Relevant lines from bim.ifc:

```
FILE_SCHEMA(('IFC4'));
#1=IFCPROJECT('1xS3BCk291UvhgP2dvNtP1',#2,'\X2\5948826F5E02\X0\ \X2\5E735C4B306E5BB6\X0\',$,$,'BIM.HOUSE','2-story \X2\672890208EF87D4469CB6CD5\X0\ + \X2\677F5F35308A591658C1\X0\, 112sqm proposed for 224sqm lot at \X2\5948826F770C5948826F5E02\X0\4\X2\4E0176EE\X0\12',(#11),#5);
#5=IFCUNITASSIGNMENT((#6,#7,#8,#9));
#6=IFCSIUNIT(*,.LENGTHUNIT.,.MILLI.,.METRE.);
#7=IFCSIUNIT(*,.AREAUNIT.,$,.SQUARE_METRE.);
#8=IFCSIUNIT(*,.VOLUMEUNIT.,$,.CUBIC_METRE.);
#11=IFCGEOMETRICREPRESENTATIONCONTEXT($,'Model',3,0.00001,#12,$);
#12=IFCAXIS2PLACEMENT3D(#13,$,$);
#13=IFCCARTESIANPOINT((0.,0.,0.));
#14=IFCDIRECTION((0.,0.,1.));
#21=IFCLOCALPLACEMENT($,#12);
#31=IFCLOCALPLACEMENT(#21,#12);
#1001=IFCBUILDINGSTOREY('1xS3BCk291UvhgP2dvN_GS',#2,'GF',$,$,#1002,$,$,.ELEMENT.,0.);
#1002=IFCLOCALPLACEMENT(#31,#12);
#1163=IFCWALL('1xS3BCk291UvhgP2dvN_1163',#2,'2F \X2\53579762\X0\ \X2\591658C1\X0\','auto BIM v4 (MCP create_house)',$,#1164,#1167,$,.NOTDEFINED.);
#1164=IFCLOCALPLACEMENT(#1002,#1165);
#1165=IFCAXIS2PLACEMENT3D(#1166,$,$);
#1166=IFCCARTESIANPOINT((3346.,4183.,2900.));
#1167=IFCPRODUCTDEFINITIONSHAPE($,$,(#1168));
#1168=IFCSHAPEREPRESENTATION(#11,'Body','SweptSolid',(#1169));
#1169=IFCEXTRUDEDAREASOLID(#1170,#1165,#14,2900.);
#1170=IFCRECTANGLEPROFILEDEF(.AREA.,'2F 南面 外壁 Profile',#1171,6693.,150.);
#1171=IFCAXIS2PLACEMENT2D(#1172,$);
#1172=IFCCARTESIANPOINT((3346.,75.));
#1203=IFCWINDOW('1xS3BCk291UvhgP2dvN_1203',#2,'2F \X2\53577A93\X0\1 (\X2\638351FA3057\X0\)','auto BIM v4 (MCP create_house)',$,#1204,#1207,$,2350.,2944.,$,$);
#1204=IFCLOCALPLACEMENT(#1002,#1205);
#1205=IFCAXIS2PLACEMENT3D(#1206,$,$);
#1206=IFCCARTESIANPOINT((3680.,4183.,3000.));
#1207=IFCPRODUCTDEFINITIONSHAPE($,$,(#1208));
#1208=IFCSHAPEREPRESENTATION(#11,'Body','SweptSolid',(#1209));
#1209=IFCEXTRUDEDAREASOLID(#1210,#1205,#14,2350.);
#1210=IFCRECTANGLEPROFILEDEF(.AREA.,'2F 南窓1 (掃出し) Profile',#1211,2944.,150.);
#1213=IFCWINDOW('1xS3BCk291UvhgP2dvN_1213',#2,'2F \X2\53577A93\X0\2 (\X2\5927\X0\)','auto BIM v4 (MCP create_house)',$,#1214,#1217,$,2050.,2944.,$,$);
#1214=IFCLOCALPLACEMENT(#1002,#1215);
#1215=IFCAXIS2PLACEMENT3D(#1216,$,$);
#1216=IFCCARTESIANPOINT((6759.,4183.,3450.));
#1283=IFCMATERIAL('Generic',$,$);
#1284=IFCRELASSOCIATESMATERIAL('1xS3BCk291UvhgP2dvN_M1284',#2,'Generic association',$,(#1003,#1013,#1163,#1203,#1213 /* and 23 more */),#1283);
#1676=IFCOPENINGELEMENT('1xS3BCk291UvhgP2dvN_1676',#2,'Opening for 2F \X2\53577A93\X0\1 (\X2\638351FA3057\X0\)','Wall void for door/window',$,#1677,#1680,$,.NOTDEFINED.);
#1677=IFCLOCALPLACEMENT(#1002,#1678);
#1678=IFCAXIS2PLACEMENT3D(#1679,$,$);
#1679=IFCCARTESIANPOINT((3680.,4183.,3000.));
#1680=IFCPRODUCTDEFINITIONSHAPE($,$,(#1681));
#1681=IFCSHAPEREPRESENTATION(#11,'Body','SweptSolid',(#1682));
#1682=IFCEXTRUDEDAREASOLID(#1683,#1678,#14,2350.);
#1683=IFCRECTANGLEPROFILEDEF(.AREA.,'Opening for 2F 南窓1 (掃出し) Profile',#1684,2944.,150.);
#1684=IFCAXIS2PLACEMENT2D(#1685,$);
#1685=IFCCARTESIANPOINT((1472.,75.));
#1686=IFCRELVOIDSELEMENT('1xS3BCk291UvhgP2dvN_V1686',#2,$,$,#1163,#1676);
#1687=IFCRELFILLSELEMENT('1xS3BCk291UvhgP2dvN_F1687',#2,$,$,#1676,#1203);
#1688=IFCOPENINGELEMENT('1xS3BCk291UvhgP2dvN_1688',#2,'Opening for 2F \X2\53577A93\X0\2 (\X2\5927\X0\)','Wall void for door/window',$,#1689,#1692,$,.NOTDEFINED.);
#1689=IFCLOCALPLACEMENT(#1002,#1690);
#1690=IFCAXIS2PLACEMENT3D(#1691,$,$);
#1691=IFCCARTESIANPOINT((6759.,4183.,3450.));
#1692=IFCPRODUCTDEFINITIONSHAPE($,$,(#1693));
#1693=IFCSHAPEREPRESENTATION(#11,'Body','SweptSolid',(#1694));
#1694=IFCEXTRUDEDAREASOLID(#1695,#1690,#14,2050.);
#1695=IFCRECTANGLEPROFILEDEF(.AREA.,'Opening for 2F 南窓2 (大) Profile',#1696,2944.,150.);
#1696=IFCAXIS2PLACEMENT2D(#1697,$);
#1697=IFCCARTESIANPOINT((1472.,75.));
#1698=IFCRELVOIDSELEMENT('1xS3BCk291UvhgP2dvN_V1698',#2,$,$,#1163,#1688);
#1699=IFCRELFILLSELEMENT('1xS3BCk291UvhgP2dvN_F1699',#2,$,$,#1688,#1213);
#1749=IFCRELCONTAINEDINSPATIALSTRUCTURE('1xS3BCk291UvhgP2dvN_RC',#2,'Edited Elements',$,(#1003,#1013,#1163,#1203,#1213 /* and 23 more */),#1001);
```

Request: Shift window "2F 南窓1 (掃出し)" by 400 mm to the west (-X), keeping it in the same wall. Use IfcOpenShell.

```python
import ifcopenshell
import ifcopenshell.api.geometry
import ifcopenshell.util.placement
import ifcopenshell.util.unit

model = ifcopenshell.open("bim.ifc")
unit_scale = ifcopenshell.util.unit.calculate_unit_scale(model)

window = model.by_guid("1xS3BCk291UvhgP2dvN_1203")
opening = window.FillsVoids[0].RelatingOpeningElement
wall = opening.VoidsElements[0].RelatingBuildingElement

wall_matrix = ifcopenshell.util.placement.get_local_placement(wall.ObjectPlacement)
shift = wall_matrix[:3, 0] * -0.4 / unit_scale
before = ifcopenshell.util.placement.get_local_placement(window.ObjectPlacement)[:3, 3].copy()

# The window is not placed relative to its opening, so move both.
for product in (opening, window):
    matrix = ifcopenshell.util.placement.get_local_placement(product.ObjectPlacement)
    matrix[:3, 3] += shift
    ifcopenshell.api.geometry.edit_object_placement(model, product=product, matrix=matrix, is_si=False)

after = ifcopenshell.util.placement.get_local_placement(window.ObjectPlacement)[:3, 3]
print("window moved by", (after - before).round(3) + 0.0)

model.write("bim_edited.ifc")
```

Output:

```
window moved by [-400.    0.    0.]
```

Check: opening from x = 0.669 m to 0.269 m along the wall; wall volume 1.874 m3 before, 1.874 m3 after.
